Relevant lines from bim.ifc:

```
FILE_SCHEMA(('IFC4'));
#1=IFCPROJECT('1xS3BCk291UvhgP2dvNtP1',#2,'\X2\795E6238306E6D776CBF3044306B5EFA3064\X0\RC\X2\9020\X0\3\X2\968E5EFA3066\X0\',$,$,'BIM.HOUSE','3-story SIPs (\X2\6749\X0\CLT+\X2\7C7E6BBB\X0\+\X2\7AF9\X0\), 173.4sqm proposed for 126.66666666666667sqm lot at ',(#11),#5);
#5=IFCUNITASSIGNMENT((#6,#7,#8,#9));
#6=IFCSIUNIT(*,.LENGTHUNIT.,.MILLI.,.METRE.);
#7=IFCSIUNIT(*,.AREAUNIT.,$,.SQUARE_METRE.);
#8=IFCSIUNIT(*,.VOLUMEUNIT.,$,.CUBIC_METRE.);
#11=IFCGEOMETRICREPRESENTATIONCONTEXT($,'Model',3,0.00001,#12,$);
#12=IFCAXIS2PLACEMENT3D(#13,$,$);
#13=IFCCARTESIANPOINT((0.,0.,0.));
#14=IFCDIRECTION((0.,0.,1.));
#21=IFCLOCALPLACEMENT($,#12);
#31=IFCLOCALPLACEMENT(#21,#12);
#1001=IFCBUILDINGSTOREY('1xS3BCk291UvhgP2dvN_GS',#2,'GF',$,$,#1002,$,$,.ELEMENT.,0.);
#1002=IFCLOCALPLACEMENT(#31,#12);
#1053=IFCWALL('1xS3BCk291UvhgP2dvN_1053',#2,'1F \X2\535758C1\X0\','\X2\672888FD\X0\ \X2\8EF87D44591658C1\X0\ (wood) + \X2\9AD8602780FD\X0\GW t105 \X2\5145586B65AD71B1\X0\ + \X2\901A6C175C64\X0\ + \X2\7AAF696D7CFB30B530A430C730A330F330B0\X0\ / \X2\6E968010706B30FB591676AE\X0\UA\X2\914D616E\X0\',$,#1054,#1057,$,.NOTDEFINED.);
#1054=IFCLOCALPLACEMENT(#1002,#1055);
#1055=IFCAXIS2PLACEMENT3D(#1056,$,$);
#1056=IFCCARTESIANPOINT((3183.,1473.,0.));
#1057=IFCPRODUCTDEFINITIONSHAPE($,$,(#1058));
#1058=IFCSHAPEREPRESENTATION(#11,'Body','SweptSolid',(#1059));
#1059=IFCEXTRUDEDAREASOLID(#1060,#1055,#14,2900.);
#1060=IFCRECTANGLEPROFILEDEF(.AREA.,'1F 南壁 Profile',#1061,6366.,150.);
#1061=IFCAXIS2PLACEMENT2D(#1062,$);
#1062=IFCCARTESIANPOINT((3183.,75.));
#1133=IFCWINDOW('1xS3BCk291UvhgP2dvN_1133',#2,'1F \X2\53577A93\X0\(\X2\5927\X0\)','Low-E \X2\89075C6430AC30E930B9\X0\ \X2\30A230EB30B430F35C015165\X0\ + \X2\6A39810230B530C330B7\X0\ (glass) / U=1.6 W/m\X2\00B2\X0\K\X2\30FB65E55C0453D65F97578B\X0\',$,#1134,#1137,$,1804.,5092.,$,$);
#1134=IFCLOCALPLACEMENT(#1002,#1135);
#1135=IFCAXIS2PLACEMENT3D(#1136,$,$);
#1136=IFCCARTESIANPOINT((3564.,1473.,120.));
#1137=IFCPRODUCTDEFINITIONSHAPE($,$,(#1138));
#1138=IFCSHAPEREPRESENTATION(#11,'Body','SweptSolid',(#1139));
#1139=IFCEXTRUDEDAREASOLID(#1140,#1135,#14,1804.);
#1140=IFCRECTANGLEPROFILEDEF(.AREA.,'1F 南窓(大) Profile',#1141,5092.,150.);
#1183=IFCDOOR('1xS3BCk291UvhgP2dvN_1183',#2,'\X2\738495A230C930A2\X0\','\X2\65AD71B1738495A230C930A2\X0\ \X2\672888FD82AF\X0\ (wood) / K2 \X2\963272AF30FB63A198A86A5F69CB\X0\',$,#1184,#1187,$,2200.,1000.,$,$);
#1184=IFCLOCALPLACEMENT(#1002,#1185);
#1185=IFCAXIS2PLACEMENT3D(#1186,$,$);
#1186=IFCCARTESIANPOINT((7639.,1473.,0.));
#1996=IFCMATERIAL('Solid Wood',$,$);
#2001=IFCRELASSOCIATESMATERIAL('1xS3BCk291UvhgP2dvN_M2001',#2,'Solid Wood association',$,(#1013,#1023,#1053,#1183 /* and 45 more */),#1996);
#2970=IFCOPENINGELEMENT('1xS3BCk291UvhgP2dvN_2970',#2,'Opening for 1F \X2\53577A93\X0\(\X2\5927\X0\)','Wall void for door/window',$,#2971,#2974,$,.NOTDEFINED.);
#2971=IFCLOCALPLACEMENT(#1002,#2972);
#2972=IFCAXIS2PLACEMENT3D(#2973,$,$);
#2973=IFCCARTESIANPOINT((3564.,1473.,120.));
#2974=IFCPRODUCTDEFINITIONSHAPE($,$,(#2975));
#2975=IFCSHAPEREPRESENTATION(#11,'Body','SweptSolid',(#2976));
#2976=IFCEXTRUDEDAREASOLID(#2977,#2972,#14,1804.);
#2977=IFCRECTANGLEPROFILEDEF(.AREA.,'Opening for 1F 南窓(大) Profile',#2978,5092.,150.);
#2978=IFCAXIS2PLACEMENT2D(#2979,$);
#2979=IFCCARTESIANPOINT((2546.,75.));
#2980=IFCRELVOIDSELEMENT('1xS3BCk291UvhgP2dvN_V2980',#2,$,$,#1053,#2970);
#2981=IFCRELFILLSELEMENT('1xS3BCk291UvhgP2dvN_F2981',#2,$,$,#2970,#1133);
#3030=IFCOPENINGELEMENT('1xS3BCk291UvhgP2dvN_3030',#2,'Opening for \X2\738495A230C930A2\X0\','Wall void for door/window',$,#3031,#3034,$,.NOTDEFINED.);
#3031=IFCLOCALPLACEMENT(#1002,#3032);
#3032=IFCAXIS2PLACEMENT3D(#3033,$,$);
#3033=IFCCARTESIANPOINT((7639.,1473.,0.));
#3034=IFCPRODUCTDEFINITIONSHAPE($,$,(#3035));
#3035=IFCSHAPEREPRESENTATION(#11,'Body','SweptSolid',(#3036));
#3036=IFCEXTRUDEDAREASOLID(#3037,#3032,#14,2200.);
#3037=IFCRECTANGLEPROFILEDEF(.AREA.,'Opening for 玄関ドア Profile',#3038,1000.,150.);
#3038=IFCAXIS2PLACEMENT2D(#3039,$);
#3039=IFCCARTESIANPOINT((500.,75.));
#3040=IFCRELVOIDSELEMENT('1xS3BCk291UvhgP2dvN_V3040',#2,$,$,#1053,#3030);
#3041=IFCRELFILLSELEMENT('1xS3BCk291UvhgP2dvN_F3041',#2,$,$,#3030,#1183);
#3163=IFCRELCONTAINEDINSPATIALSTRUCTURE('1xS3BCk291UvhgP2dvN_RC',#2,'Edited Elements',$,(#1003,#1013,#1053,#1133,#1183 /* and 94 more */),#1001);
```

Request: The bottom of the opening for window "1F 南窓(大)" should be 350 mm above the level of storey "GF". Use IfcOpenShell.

```python
import numpy as np
import ifcopenshell
import ifcopenshell.api.geometry
import ifcopenshell.geom
import ifcopenshell.util.element
import ifcopenshell.util.placement
import ifcopenshell.util.shape
import ifcopenshell.util.unit

model = ifcopenshell.open("bim.ifc")
unit_scale = ifcopenshell.util.unit.calculate_unit_scale(model)

window = model.by_id(1133)
opening = window.FillsVoids[0].RelatingOpeningElement
storey = ifcopenshell.util.element.get_container(window, ifc_class="IfcBuildingStorey")
level = ifcopenshell.util.placement.get_local_placement(storey.ObjectPlacement)[2, 3]

# The opening's origin need not be at the sill, so measure its lowest point.
shape = ifcopenshell.geom.create_shape(ifcopenshell.geom.settings(), opening)
bottom = ifcopenshell.util.shape.get_shape_bottom_elevation(shape, shape.geometry) / unit_scale
dz = level + 0.35 / unit_scale - bottom

shift = np.array([0.0, 0.0, dz])
# The window is not placed relative to its opening, so move both.
for product in (opening, window):
    matrix = ifcopenshell.util.placement.get_local_placement(product.ObjectPlacement)
    matrix[:3, 3] += shift
    ifcopenshell.api.geometry.edit_object_placement(model, product=product, matrix=matrix, is_si=False)

print(f"moved by {dz * unit_scale:+.3f} m")

model.write("bim_v2.ifc")
```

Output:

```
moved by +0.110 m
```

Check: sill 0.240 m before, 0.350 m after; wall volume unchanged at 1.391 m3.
